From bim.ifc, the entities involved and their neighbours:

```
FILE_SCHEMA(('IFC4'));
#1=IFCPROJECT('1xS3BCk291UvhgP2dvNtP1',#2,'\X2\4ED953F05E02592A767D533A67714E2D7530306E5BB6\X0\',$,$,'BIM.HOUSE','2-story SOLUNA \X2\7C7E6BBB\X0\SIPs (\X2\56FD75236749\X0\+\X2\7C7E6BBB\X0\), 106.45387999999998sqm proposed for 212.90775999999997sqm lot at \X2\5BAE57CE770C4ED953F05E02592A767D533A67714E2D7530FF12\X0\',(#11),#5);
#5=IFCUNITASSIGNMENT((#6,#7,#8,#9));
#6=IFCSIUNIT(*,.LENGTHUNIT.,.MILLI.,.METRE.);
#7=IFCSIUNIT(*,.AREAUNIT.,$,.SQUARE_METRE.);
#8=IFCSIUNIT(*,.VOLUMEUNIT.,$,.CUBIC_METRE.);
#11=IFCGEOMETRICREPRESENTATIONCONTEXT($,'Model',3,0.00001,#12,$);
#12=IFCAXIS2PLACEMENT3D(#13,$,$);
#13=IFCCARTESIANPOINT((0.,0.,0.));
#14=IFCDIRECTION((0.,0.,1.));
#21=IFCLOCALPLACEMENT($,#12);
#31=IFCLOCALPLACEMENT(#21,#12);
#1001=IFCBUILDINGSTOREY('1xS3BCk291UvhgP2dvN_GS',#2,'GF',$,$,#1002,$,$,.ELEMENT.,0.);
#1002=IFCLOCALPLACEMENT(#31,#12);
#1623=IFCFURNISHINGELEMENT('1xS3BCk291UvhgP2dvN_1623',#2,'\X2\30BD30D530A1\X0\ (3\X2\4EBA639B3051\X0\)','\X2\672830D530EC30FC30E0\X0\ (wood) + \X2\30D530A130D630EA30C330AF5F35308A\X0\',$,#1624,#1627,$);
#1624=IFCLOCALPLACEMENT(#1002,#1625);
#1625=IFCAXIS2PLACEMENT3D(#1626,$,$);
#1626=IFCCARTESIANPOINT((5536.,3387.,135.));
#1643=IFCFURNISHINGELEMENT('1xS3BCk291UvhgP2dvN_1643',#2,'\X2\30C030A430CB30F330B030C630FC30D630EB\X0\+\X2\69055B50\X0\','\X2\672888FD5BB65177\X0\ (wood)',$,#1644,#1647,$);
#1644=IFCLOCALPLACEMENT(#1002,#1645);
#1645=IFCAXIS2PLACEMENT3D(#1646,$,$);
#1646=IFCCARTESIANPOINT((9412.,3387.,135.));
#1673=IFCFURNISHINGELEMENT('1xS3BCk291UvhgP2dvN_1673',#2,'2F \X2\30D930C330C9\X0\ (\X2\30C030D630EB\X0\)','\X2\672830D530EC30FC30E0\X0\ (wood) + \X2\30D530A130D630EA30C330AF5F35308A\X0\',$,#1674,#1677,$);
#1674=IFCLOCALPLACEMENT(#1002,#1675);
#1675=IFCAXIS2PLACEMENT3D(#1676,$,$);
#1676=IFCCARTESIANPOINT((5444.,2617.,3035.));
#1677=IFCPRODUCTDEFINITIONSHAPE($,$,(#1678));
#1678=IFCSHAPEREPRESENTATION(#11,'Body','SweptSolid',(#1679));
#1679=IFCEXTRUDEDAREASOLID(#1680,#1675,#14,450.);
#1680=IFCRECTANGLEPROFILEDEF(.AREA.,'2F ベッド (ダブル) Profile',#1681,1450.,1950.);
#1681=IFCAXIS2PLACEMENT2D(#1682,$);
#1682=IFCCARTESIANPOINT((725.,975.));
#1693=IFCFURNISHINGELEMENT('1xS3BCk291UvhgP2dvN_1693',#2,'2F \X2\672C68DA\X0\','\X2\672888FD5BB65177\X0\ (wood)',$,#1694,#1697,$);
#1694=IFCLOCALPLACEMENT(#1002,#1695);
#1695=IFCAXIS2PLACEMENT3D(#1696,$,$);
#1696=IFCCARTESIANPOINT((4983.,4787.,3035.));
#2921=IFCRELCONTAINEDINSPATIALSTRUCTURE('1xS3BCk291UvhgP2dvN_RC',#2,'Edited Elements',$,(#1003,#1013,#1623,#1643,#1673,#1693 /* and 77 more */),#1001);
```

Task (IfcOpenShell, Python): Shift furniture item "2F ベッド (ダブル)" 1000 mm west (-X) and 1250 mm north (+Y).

```python
import ifcopenshell
import ifcopenshell.api.geometry
import ifcopenshell.util.placement
import ifcopenshell.util.unit

model = ifcopenshell.open("bim.ifc")
unit_scale = ifcopenshell.util.unit.calculate_unit_scale(model)

item = model.by_guid("1xS3BCk291UvhgP2dvN_1673")
matrix = ifcopenshell.util.placement.get_local_placement(item.ObjectPlacement)
matrix[0, 3] -= 1 / unit_scale
matrix[1, 3] += 1.25 / unit_scale
ifcopenshell.api.geometry.edit_object_placement(model, product=item, matrix=matrix, is_si=False)

print(ifcopenshell.util.placement.get_local_placement(item.ObjectPlacement).round(3) + 0.0)

model.write("bim_updated.ifc")
```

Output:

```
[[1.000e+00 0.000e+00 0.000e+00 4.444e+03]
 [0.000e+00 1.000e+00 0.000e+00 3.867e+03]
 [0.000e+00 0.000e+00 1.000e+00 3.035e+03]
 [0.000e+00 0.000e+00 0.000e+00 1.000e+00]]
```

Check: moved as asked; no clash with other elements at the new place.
